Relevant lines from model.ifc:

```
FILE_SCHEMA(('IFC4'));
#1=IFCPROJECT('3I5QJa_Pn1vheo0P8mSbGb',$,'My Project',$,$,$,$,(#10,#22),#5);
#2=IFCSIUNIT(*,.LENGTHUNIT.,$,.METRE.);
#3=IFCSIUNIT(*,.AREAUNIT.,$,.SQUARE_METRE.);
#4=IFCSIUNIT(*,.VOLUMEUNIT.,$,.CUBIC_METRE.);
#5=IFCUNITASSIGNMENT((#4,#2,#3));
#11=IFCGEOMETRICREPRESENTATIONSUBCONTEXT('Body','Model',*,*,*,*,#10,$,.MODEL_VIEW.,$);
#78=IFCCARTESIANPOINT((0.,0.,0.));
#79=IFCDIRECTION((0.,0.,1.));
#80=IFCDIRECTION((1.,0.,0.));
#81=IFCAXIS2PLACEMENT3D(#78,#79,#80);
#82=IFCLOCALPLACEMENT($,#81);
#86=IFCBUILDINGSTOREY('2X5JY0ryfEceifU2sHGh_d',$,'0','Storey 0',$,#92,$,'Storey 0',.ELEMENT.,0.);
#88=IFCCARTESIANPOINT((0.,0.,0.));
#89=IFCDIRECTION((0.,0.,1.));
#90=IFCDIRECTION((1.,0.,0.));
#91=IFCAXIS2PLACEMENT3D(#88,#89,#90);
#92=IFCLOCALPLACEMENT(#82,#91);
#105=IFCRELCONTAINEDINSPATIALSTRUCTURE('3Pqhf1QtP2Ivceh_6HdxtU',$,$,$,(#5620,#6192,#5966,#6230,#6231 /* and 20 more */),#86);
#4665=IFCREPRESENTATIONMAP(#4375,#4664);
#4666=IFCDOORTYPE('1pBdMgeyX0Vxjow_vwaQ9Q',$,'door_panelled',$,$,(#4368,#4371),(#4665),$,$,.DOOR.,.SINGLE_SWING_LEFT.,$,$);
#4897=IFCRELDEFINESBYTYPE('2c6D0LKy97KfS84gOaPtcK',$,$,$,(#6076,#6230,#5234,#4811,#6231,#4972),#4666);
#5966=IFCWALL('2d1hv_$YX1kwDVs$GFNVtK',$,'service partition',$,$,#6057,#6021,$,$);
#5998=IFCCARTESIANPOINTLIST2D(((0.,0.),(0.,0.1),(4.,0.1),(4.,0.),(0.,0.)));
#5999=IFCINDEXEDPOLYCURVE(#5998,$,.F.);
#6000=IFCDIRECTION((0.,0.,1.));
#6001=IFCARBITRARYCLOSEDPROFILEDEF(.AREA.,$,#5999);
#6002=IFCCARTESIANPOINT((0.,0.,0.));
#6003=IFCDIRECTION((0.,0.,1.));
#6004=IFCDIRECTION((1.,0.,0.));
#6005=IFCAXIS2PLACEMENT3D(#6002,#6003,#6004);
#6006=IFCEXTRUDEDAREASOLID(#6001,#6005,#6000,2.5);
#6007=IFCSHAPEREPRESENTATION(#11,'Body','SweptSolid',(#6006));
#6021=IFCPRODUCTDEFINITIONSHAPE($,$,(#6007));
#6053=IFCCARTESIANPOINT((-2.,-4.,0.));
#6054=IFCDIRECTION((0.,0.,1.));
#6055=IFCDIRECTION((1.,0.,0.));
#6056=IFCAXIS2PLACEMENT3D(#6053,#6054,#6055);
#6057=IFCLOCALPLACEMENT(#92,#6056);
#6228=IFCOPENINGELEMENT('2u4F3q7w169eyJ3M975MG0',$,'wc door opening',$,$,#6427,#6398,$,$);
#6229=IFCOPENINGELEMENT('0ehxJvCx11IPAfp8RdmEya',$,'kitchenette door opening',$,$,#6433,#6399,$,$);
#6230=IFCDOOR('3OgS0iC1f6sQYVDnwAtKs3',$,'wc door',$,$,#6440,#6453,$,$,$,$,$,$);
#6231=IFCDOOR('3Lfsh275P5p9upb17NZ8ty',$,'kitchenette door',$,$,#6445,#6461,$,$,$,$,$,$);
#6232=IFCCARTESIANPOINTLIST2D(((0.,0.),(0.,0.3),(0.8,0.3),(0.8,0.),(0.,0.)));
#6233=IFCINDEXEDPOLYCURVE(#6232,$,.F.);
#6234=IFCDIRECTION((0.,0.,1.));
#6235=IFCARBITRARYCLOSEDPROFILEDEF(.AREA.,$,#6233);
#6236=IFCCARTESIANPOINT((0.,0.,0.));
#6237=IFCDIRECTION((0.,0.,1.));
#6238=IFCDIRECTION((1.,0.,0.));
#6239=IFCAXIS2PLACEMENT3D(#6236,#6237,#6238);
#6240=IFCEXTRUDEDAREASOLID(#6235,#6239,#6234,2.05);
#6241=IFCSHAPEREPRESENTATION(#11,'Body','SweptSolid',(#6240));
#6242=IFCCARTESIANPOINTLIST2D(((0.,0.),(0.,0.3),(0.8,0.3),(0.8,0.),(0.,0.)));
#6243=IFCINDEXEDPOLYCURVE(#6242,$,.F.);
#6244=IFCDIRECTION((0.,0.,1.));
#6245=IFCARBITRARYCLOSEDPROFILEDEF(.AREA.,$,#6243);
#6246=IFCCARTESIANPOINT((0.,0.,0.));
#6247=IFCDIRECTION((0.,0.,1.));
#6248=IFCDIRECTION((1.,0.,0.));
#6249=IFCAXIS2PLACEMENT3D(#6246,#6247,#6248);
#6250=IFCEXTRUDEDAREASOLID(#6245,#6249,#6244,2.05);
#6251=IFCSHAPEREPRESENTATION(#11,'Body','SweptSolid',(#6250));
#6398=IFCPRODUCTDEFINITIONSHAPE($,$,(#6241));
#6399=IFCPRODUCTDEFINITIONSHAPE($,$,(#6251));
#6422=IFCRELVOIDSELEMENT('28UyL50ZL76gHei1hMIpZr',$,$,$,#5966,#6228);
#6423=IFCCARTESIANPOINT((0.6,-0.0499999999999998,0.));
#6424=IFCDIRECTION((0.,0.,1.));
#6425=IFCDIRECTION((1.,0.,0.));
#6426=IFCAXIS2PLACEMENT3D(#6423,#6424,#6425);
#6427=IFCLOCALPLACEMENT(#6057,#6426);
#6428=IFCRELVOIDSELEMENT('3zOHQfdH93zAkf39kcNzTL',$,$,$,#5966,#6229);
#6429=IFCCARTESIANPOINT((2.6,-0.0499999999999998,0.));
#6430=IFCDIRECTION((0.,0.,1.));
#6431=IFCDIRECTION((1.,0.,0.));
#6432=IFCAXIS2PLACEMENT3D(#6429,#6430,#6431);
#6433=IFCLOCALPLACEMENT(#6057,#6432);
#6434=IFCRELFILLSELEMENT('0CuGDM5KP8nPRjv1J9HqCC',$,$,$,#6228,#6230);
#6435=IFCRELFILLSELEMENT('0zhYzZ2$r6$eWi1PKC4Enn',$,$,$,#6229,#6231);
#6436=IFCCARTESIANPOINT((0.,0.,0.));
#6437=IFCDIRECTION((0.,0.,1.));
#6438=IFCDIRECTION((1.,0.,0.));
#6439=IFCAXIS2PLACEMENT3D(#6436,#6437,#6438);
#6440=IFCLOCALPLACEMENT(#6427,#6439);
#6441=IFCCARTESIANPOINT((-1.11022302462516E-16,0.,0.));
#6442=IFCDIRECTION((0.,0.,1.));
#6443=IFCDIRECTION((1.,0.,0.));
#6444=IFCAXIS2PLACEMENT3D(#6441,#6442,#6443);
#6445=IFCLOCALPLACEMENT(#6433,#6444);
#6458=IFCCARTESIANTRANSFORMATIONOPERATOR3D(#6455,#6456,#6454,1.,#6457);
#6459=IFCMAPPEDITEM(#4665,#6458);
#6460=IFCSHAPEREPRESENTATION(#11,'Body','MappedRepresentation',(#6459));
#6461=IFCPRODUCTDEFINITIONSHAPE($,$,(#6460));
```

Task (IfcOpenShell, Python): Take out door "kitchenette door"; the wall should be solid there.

```python
import ifcopenshell
import ifcopenshell.api.feature
import ifcopenshell.api.root
import ifcopenshell.geom
import ifcopenshell.util.shape

model = ifcopenshell.open("model.ifc")
settings = ifcopenshell.geom.settings()


def volume(element):
    """Net volume in cubic metres, openings subtracted."""
    shape = ifcopenshell.geom.create_shape(settings, element)
    return ifcopenshell.util.shape.get_volume(shape.geometry)


door = model.by_guid("3Lfsh275P5p9upb17NZ8ty")
opening = door.FillsVoids[0].RelatingOpeningElement
wall = opening.VoidsElements[0].RelatingBuildingElement
before = volume(wall)

ifcopenshell.api.root.remove_product(model, product=door)
ifcopenshell.api.feature.remove_feature(model, feature=opening)

after = volume(wall)

print(f"wall volume {before:.3f} -> {after:.3f} m3")

model.write("model-out.ifc")
```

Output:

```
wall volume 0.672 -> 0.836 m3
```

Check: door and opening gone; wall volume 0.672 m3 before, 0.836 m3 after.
